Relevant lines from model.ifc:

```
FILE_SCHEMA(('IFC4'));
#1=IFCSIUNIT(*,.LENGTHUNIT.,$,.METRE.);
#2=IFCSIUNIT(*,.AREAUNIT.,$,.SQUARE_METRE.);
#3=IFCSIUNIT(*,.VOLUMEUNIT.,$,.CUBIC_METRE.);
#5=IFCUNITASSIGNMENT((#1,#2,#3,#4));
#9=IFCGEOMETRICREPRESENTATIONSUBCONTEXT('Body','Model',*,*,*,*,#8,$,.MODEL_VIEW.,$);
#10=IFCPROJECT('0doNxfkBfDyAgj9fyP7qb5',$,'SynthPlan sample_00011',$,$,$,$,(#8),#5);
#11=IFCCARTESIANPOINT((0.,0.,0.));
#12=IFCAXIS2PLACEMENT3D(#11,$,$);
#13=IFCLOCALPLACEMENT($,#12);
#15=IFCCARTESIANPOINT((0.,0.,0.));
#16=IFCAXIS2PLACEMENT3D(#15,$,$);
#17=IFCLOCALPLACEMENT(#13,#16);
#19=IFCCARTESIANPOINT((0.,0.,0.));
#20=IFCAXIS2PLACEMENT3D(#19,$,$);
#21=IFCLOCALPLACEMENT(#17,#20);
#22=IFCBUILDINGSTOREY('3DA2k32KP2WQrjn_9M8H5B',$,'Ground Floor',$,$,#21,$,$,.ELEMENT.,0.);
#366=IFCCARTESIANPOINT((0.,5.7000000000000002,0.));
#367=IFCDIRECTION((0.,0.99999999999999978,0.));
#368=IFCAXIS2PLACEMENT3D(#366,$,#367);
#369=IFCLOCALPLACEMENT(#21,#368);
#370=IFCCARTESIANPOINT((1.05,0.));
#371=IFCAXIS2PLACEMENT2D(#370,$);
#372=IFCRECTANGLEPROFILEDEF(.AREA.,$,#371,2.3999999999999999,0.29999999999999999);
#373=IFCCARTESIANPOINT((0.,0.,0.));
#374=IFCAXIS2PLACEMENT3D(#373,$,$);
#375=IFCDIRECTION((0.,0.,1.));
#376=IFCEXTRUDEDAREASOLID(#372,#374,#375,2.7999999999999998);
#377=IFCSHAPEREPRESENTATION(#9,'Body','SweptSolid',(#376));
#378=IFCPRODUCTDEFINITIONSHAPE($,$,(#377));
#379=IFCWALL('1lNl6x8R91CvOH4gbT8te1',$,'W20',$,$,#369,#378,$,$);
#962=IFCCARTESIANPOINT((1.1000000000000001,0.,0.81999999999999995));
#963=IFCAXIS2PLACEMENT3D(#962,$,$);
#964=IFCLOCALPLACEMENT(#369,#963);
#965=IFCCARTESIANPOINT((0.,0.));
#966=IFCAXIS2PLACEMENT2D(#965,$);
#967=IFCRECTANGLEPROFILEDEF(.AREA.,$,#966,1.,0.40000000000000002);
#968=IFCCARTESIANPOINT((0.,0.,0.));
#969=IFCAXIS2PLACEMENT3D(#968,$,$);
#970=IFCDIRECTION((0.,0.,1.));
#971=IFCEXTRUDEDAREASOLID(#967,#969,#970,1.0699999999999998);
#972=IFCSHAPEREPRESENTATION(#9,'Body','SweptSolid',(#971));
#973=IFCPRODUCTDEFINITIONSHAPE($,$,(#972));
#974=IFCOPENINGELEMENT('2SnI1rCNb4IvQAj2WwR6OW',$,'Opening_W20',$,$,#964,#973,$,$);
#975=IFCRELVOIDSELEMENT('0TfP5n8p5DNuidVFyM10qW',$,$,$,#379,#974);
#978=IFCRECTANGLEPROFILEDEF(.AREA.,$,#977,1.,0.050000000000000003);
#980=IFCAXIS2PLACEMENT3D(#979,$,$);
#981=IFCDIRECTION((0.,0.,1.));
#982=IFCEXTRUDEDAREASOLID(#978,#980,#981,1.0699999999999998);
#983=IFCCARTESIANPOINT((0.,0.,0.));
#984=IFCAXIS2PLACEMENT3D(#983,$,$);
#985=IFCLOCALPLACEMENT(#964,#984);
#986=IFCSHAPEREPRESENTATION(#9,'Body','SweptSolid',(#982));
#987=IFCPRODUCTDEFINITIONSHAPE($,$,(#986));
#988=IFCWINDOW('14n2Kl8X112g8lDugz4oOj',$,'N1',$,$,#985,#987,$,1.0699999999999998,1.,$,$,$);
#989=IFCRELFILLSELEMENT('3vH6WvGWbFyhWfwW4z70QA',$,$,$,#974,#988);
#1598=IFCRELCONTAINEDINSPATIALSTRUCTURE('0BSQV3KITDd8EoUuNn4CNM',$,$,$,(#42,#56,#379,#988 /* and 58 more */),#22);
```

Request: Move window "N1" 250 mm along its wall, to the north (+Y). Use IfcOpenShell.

```python
import ifcopenshell
import ifcopenshell.api.geometry
import ifcopenshell.util.placement

model = ifcopenshell.open("model.ifc")

window = model.by_guid("14n2Kl8X112g8lDugz4oOj")
opening = window.FillsVoids[0].RelatingOpeningElement
wall = opening.VoidsElements[0].RelatingBuildingElement

wall_matrix = ifcopenshell.util.placement.get_local_placement(wall.ObjectPlacement)
shift = wall_matrix[:3, 0] * 0.25
before = ifcopenshell.util.placement.get_local_placement(window.ObjectPlacement)[:3, 3].copy()

# The window is placed relative to its opening, so it follows when the opening moves.
matrix = ifcopenshell.util.placement.get_local_placement(opening.ObjectPlacement)
matrix[:3, 3] += shift
ifcopenshell.api.geometry.edit_object_placement(
    model, product=opening, matrix=matrix, is_si=False, should_transform_children=True
)

after = ifcopenshell.util.placement.get_local_placement(window.ObjectPlacement)[:3, 3]
print("window moved by", (after - before).round(3) + 0.0)

model.write("model_v2.ifc")
```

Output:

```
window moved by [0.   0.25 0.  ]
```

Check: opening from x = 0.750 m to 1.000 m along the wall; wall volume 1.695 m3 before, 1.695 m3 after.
